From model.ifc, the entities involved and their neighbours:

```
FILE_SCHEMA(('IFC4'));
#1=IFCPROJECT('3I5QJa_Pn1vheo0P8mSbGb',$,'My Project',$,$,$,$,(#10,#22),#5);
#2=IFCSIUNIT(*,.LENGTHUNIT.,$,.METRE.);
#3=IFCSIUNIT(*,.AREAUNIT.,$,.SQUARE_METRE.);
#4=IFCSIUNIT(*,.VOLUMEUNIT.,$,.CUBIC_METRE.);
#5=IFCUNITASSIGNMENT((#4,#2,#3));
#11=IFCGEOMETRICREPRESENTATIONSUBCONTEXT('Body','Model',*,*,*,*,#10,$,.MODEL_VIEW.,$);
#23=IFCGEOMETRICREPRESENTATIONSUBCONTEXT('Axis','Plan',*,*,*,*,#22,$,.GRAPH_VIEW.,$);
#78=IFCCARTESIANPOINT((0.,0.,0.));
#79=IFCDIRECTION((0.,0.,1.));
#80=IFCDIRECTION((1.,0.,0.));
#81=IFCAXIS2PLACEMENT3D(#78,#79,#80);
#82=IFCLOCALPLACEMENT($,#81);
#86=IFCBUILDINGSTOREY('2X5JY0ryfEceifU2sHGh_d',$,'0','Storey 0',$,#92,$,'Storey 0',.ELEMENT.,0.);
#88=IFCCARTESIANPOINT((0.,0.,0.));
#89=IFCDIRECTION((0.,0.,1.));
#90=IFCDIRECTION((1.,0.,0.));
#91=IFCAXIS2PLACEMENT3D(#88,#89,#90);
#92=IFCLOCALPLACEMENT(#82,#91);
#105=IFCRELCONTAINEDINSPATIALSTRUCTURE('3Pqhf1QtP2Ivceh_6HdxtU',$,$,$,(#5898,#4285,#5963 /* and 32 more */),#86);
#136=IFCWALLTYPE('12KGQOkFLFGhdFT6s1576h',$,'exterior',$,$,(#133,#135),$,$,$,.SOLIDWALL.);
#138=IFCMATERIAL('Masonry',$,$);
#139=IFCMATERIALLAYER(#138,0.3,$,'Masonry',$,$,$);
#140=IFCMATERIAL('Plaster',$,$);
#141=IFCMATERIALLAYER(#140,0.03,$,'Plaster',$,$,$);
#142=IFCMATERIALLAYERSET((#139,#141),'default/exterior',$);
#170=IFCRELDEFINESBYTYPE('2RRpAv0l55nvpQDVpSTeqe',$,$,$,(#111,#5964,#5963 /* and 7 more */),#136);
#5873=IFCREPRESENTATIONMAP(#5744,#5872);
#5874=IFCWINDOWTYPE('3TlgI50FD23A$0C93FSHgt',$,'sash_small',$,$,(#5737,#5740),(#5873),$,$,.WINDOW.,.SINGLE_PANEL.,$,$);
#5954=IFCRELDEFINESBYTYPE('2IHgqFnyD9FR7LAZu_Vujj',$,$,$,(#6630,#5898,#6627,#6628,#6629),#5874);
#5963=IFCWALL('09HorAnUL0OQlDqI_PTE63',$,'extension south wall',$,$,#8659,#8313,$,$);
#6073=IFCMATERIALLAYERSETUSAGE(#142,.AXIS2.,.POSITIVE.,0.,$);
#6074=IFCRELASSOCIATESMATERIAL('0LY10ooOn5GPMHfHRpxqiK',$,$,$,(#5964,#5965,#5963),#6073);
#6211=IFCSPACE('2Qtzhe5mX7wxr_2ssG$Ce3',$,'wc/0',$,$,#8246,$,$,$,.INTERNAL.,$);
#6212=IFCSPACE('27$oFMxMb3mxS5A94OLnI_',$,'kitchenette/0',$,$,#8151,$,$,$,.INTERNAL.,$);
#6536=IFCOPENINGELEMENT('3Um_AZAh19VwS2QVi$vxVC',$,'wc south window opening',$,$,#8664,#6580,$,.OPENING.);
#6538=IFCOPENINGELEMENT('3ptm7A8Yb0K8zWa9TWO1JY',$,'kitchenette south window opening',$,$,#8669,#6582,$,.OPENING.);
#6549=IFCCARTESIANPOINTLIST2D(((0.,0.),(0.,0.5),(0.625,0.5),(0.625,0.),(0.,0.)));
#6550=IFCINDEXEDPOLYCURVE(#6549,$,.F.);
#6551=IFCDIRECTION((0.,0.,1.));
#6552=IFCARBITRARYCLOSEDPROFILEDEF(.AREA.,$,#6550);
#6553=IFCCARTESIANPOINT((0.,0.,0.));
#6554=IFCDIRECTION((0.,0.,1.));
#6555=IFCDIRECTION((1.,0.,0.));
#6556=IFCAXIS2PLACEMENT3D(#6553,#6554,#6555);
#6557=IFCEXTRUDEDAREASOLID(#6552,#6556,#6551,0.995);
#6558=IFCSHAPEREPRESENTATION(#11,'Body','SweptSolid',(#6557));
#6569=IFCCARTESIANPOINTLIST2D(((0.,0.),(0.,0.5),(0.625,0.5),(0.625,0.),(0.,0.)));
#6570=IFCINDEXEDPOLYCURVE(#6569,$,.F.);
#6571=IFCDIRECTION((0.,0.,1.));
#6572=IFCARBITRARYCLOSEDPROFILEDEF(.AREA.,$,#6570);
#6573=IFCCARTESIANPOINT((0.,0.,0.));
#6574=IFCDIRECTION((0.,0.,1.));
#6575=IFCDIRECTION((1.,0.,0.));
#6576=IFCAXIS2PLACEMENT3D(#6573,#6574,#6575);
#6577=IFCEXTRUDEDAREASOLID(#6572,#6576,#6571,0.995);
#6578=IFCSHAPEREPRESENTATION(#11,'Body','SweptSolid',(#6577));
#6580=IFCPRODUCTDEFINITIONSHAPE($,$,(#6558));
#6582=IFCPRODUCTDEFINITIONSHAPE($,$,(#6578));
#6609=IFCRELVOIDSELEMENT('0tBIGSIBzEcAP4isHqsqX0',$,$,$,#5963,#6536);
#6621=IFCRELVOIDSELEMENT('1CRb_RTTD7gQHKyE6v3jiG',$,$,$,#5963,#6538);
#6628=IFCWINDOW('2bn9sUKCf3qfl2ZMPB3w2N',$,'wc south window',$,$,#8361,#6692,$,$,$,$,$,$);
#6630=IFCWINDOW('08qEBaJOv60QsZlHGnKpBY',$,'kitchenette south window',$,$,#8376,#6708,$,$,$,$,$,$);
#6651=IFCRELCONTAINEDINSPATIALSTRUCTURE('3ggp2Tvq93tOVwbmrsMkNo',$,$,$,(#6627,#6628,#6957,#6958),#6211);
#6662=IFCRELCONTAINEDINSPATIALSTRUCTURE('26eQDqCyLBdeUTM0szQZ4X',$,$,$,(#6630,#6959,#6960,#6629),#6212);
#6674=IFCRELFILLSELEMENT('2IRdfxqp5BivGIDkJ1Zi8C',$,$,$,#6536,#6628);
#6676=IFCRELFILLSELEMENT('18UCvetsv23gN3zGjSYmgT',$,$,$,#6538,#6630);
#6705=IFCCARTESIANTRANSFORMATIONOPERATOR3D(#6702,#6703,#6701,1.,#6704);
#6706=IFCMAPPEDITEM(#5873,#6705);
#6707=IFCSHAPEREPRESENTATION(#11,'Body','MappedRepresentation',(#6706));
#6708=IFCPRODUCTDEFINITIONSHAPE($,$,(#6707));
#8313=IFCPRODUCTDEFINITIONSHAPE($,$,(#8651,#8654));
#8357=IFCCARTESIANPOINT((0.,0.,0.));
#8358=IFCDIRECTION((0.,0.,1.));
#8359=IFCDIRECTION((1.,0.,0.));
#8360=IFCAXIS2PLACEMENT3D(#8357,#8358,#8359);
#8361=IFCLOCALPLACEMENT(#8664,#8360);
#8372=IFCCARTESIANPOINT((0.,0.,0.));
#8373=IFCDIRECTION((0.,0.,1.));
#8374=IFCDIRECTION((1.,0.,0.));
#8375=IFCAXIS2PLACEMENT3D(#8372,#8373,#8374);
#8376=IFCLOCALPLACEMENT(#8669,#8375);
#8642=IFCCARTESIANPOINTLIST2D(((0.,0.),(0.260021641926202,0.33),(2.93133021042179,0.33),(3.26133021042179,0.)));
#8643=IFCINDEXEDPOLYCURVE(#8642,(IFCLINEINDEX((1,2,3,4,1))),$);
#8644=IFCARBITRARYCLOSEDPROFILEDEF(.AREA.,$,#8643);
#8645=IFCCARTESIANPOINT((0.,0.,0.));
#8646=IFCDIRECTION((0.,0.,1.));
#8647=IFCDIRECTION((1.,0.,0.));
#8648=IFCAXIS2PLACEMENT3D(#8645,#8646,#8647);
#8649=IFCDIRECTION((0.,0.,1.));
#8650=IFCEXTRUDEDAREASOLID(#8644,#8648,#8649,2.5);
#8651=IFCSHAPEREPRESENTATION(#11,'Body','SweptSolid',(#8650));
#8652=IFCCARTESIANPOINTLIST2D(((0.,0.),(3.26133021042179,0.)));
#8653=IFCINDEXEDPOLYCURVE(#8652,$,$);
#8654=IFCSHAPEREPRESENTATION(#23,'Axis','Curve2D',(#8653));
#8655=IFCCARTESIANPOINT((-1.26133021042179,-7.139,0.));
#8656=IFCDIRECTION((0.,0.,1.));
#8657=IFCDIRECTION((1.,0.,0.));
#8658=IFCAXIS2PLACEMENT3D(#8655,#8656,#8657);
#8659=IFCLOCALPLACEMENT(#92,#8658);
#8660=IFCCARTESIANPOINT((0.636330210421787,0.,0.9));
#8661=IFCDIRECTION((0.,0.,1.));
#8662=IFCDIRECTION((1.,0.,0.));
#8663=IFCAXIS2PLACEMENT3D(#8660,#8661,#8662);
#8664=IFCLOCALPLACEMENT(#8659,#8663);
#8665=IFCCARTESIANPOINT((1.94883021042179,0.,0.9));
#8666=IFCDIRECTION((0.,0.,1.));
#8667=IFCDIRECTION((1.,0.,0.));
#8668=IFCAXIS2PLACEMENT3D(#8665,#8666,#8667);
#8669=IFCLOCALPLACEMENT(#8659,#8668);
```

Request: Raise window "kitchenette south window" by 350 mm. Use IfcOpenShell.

```python
import numpy as np
import ifcopenshell
import ifcopenshell.api.geometry
import ifcopenshell.util.placement
import ifcopenshell.util.unit

model = ifcopenshell.open("model.ifc")
unit_scale = ifcopenshell.util.unit.calculate_unit_scale(model)

window = model.by_id(6630)
opening = window.FillsVoids[0].RelatingOpeningElement
dz = 0.35 / unit_scale

shift = np.array([0.0, 0.0, dz])
# The window is placed relative to its opening, so it follows when the opening moves.
matrix = ifcopenshell.util.placement.get_local_placement(opening.ObjectPlacement)
matrix[:3, 3] += shift
ifcopenshell.api.geometry.edit_object_placement(
    model, product=opening, matrix=matrix, is_si=False, should_transform_children=True
)

print(f"moved by {dz * unit_scale:+.3f} m")

model.write("model_rev.ifc")
```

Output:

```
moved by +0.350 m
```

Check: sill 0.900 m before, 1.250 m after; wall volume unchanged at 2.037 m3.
